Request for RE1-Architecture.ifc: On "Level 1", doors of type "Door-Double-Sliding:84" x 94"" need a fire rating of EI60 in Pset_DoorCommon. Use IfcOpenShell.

First a look at what the model holds.

```python
import ifcopenshell
import ifcopenshell.util.element

model = ifcopenshell.open("RE1-Architecture.ifc")
print(model.schema)
storey = next(s for s in model.by_type("IfcBuildingStorey") if s.Name == "Level 1")
doors = [e for e in ifcopenshell.util.element.get_decomposition(storey) if e.is_a("IfcDoor")]
seen = {}
for e in doors:
    element_type = ifcopenshell.util.element.get_type(e)
    key = (element_type.Name if element_type != e and element_type else None, ifcopenshell.util.element.get_pset(e, "Pset_DoorCommon", "FireRating"))
    seen[key] = seen.get(key, 0) + 1
for (name, value), count in sorted(seen.items(), key=str):
    print(count, "x", name, "|", value)
```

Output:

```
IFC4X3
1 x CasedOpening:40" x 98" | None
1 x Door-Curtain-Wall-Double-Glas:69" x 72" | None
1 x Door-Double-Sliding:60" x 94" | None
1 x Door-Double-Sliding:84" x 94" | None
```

```python
import ifcopenshell
import ifcopenshell.api.pset
import ifcopenshell.util.element

model = ifcopenshell.open("RE1-Architecture.ifc")

storey = next(s for s in model.by_type("IfcBuildingStorey") if s.Name == "Level 1")
doors = [e for e in ifcopenshell.util.element.get_decomposition(storey) if e.is_a("IfcDoor")]

count = 0
for e in doors:
    element_type = ifcopenshell.util.element.get_type(e)
    if element_type in (None, e) or element_type.Name != 'Door-Double-Sliding:84" x 94"':
        continue
    # add_pset returns the element's existing set when there is one.
    pset = ifcopenshell.api.pset.add_pset(model, product=e, name="Pset_DoorCommon")
    ifcopenshell.api.pset.edit_pset(model, pset=pset, properties={"FireRating": "EI60"})
    count += 1

print(count, "doors updated")

model.write("RE1-Architecture_v2.ifc")
```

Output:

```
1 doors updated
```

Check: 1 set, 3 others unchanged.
